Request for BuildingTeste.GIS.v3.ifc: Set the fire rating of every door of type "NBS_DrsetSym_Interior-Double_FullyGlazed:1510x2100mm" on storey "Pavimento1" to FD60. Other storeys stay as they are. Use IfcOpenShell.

First a look at what the model holds.

```python
import ifcopenshell
import ifcopenshell.util.element

model = ifcopenshell.open("BuildingTeste.GIS.v3.ifc")
print(model.schema)
storey = next(s for s in model.by_type("IfcBuildingStorey") if s.Name == "Pavimento1")
doors = [e for e in ifcopenshell.util.element.get_decomposition(storey) if e.is_a("IfcDoor")]
seen = {}
for e in doors:
    element_type = ifcopenshell.util.element.get_type(e)
    key = (element_type.Name if element_type != e and element_type else None, ifcopenshell.util.element.get_pset(e, "Pset_DoorCommon", "FireRating"))
    seen[key] = seen.get(key, 0) + 1
for (name, value), count in sorted(seen.items(), key=str):
    print(count, "x", name, "|", value)
```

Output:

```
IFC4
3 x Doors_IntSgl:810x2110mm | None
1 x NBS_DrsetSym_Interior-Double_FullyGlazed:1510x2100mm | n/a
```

```python
import ifcopenshell
import ifcopenshell.api.pset
import ifcopenshell.util.element

model = ifcopenshell.open("BuildingTeste.GIS.v3.ifc")

storey = next(s for s in model.by_type("IfcBuildingStorey") if s.Name == "Pavimento1")
doors = [e for e in ifcopenshell.util.element.get_decomposition(storey) if e.is_a("IfcDoor")]

count = 0
for e in doors:
    element_type = ifcopenshell.util.element.get_type(e)
    if element_type in (None, e) or element_type.Name != "NBS_DrsetSym_Interior-Double_FullyGlazed:1510x2100mm":
        continue
    # add_pset returns the element's existing set when there is one.
    pset = ifcopenshell.api.pset.add_pset(model, product=e, name="Pset_DoorCommon")
    ifcopenshell.api.pset.edit_pset(model, pset=pset, properties={"FireRating": "FD60"})
    count += 1

print(count, "doors updated")

model.write("BuildingTeste.GIS.v3_v2.ifc")
```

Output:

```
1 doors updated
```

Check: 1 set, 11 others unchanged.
